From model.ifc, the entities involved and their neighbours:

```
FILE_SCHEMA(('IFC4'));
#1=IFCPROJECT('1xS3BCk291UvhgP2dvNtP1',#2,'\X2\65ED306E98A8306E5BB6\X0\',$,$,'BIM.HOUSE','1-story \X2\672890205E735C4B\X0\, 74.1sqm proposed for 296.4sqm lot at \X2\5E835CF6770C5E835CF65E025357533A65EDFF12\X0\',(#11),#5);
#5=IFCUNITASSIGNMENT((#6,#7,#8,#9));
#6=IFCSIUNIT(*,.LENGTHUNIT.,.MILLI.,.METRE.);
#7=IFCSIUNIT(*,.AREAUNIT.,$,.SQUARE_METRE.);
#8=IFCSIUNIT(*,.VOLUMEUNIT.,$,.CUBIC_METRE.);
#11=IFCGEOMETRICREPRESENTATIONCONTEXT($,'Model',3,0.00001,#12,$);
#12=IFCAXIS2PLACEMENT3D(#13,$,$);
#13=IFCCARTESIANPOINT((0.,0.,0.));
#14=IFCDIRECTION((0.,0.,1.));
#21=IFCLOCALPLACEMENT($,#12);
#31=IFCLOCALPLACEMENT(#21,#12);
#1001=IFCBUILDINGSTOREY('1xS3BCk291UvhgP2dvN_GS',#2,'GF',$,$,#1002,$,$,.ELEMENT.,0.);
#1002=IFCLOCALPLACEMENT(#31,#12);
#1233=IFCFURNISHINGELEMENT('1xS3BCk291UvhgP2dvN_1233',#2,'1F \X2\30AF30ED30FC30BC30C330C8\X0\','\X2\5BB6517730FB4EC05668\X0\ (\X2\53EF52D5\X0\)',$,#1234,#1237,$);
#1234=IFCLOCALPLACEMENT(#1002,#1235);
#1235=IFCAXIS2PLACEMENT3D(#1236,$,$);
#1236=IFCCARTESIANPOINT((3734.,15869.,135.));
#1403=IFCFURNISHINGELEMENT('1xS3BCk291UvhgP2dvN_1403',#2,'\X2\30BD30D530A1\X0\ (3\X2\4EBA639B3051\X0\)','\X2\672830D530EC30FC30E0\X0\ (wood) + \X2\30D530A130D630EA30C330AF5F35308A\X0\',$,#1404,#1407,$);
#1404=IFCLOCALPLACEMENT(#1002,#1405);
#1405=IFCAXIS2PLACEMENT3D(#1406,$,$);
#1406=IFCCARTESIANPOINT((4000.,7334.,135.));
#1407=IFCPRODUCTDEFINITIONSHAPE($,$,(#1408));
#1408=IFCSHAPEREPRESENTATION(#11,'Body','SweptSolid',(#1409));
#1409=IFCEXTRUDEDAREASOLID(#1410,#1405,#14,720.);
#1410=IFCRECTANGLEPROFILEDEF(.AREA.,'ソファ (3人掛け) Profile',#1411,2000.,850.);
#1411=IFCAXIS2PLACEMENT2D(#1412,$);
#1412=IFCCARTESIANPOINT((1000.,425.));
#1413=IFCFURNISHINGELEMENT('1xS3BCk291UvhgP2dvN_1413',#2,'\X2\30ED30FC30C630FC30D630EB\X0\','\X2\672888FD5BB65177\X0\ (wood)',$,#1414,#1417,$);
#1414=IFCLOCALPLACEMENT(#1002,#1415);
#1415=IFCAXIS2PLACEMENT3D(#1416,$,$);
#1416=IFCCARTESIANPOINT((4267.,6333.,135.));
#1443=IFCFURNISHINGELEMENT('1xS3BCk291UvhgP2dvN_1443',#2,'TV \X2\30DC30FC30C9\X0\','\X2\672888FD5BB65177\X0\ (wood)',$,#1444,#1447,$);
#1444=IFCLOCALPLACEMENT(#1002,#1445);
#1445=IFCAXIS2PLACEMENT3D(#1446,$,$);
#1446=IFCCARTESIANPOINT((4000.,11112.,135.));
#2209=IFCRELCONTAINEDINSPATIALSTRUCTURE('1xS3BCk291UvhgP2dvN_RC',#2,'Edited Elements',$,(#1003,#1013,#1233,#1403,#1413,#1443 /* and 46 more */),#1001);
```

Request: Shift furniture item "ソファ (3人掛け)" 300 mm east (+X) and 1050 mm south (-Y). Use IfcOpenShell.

```python
import ifcopenshell
import ifcopenshell.api.geometry
import ifcopenshell.util.placement
import ifcopenshell.util.unit

model = ifcopenshell.open("model.ifc")
unit_scale = ifcopenshell.util.unit.calculate_unit_scale(model)

item = model.by_guid("1xS3BCk291UvhgP2dvN_1403")
matrix = ifcopenshell.util.placement.get_local_placement(item.ObjectPlacement)
matrix[0, 3] += 0.3 / unit_scale
matrix[1, 3] -= 1.05 / unit_scale
ifcopenshell.api.geometry.edit_object_placement(model, product=item, matrix=matrix, is_si=False)

print(ifcopenshell.util.placement.get_local_placement(item.ObjectPlacement).round(3) + 0.0)

model.write("model_rev.ifc")
```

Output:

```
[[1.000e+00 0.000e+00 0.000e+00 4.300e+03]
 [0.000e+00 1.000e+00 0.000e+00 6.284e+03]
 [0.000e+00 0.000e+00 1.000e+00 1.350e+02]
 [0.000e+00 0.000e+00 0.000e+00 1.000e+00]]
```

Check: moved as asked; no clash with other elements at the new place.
